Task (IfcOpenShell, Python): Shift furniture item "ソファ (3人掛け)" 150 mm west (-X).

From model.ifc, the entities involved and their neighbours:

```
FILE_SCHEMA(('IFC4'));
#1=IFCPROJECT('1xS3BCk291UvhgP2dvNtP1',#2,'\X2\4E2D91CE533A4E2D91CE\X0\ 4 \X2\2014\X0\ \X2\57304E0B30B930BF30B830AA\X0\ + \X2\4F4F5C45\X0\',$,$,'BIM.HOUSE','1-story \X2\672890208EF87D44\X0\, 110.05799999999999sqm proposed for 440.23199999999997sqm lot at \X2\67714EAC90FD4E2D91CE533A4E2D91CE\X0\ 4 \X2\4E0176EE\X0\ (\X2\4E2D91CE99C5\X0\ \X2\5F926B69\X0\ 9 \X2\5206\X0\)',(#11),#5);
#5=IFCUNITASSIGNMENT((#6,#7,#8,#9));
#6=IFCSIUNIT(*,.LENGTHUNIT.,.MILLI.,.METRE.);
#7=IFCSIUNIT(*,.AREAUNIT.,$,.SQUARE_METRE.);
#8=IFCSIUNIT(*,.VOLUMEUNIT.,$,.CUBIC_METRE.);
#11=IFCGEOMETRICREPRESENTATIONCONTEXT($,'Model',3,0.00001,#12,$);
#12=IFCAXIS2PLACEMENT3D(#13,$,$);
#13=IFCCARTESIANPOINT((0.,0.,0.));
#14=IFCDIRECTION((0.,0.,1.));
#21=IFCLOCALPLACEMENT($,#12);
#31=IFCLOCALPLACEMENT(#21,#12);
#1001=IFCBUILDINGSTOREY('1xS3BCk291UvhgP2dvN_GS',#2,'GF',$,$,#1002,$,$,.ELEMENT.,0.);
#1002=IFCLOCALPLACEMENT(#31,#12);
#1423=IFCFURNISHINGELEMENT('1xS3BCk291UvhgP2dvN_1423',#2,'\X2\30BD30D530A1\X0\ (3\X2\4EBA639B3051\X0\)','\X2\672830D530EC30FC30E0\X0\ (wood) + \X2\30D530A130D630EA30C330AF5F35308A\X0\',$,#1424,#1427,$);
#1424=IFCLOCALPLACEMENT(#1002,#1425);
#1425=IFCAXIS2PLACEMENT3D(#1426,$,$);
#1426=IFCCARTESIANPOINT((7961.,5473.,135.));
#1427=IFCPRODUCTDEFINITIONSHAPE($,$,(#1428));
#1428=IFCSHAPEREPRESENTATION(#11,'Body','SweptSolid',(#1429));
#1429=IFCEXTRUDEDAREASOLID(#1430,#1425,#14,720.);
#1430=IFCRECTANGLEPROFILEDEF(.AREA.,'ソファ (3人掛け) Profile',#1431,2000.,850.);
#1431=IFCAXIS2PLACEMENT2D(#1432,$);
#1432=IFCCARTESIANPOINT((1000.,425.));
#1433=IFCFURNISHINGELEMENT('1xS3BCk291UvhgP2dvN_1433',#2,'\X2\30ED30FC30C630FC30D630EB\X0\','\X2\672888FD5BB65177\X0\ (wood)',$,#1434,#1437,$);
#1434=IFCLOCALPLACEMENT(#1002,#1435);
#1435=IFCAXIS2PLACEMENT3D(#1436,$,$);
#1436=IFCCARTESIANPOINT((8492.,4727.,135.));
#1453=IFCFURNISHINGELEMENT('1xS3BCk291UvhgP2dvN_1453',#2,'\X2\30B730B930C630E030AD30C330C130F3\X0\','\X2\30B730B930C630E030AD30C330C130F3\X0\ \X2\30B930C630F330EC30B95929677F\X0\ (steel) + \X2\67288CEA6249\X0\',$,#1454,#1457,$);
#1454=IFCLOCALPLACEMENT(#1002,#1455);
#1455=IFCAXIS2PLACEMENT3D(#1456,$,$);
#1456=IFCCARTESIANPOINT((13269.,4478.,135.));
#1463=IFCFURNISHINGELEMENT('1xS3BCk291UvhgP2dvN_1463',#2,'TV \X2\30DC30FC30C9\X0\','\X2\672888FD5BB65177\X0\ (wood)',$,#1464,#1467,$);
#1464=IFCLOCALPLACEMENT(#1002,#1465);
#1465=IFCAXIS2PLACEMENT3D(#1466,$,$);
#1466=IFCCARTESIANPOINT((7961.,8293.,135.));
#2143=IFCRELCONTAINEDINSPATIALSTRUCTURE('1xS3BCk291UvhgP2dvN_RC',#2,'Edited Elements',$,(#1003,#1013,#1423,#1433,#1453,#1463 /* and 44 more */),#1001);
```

```python
import ifcopenshell
import ifcopenshell.api.geometry
import ifcopenshell.util.placement
import ifcopenshell.util.unit

model = ifcopenshell.open("model.ifc")
unit_scale = ifcopenshell.util.unit.calculate_unit_scale(model)

item = model.by_id(1423)
matrix = ifcopenshell.util.placement.get_local_placement(item.ObjectPlacement)
matrix[0, 3] -= 0.15 / unit_scale
ifcopenshell.api.geometry.edit_object_placement(model, product=item, matrix=matrix, is_si=False)

print(ifcopenshell.util.placement.get_local_placement(item.ObjectPlacement).round(3) + 0.0)

model.write("model_updated.ifc")
```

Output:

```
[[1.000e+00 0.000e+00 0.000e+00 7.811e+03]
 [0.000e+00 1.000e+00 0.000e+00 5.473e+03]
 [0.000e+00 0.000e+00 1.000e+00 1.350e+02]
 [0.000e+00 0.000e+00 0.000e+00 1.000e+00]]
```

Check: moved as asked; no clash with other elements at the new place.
